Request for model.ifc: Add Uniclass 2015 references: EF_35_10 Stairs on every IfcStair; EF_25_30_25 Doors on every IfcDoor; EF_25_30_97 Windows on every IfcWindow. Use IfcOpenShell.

First a look at what the model holds.

```python
import ifcopenshell

model = ifcopenshell.open("model.ifc")
print(model.schema)
print("classifications:", [c.Name for c in model.by_type("IfcClassification")])
for ifc_class in ("IfcDoor", "IfcRoof", "IfcStair", "IfcWall", "IfcWindow"):
    print(ifc_class, len(model.by_type(ifc_class)))
```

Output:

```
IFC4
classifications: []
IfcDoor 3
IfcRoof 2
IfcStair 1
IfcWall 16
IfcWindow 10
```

```python
import ifcopenshell
import ifcopenshell.api.classification

model = ifcopenshell.open("model.ifc")

system = ifcopenshell.api.classification.add_classification(model, classification="Uniclass 2015")

codes = {
    "IfcStair": ("EF_35_10", "Stairs"),
    "IfcDoor": ("EF_25_30_25", "Doors"),
    "IfcWindow": ("EF_25_30_97", "Windows"),
}
for ifc_class, (code, name) in codes.items():
    products = model.by_type(ifc_class)
    ifcopenshell.api.classification.add_reference(
        model, products=products, classification=system, identification=code, name=name
    )
    print(code, len(products))

model.write("model_v2.ifc")
```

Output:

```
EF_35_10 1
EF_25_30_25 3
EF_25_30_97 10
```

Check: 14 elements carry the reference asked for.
